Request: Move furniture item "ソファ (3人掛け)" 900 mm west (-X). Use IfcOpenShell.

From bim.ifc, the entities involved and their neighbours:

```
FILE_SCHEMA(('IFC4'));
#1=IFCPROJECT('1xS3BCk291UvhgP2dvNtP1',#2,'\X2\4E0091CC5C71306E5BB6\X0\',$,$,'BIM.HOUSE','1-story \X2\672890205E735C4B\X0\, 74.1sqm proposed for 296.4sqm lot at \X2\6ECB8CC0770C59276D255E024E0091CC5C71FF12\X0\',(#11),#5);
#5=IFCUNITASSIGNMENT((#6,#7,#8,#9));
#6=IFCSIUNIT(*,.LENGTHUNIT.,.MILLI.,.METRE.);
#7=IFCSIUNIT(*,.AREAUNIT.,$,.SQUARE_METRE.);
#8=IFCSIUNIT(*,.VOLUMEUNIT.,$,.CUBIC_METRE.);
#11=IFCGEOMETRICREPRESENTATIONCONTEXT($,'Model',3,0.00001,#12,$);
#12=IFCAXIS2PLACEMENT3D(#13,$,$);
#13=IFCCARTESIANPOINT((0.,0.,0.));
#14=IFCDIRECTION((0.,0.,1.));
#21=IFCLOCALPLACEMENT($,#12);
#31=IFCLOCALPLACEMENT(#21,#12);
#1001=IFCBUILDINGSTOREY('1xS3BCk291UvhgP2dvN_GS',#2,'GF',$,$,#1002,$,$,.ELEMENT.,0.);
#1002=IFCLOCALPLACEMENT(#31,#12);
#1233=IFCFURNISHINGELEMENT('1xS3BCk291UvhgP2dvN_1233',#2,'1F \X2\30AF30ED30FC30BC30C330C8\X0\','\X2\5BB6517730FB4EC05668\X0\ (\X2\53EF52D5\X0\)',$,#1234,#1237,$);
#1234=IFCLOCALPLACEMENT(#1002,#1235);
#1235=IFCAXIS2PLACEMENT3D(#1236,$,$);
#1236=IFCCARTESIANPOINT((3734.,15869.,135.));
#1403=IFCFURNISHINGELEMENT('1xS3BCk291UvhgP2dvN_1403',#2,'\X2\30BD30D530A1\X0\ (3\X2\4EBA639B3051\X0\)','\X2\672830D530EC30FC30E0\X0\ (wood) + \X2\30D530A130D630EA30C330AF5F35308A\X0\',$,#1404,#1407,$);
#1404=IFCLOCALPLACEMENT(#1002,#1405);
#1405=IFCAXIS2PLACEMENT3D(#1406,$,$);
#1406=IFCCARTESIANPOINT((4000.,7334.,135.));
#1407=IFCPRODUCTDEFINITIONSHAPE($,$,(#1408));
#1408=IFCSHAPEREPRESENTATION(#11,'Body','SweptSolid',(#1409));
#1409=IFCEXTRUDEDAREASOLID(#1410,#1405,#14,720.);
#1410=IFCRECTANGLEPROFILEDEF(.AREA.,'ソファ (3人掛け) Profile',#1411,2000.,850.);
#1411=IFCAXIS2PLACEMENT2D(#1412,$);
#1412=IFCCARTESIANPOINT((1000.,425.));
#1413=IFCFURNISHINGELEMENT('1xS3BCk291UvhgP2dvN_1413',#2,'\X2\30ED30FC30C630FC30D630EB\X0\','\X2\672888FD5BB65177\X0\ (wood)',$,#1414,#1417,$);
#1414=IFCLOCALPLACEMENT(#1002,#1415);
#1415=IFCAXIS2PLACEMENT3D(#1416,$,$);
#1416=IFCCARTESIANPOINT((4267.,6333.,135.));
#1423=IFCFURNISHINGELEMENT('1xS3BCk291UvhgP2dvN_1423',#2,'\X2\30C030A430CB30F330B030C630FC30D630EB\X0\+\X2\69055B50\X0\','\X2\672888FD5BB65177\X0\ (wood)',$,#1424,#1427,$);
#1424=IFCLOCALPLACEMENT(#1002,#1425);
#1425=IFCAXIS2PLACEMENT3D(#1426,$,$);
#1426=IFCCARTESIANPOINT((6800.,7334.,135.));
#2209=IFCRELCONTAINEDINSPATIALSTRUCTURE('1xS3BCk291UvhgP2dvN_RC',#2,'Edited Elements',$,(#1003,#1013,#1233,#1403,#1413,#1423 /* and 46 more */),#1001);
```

```python
import ifcopenshell
import ifcopenshell.api.geometry
import ifcopenshell.util.placement
import ifcopenshell.util.unit

model = ifcopenshell.open("bim.ifc")
unit_scale = ifcopenshell.util.unit.calculate_unit_scale(model)

item = model.by_id(1403)
matrix = ifcopenshell.util.placement.get_local_placement(item.ObjectPlacement)
matrix[0, 3] -= 0.9 / unit_scale
ifcopenshell.api.geometry.edit_object_placement(model, product=item, matrix=matrix, is_si=False)

print(ifcopenshell.util.placement.get_local_placement(item.ObjectPlacement).round(3) + 0.0)

model.write("bim_rev.ifc")
```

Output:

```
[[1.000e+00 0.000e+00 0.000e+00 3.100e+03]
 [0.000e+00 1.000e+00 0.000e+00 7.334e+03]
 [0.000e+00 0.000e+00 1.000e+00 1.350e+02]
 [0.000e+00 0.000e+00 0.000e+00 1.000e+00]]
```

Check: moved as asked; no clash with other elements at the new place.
